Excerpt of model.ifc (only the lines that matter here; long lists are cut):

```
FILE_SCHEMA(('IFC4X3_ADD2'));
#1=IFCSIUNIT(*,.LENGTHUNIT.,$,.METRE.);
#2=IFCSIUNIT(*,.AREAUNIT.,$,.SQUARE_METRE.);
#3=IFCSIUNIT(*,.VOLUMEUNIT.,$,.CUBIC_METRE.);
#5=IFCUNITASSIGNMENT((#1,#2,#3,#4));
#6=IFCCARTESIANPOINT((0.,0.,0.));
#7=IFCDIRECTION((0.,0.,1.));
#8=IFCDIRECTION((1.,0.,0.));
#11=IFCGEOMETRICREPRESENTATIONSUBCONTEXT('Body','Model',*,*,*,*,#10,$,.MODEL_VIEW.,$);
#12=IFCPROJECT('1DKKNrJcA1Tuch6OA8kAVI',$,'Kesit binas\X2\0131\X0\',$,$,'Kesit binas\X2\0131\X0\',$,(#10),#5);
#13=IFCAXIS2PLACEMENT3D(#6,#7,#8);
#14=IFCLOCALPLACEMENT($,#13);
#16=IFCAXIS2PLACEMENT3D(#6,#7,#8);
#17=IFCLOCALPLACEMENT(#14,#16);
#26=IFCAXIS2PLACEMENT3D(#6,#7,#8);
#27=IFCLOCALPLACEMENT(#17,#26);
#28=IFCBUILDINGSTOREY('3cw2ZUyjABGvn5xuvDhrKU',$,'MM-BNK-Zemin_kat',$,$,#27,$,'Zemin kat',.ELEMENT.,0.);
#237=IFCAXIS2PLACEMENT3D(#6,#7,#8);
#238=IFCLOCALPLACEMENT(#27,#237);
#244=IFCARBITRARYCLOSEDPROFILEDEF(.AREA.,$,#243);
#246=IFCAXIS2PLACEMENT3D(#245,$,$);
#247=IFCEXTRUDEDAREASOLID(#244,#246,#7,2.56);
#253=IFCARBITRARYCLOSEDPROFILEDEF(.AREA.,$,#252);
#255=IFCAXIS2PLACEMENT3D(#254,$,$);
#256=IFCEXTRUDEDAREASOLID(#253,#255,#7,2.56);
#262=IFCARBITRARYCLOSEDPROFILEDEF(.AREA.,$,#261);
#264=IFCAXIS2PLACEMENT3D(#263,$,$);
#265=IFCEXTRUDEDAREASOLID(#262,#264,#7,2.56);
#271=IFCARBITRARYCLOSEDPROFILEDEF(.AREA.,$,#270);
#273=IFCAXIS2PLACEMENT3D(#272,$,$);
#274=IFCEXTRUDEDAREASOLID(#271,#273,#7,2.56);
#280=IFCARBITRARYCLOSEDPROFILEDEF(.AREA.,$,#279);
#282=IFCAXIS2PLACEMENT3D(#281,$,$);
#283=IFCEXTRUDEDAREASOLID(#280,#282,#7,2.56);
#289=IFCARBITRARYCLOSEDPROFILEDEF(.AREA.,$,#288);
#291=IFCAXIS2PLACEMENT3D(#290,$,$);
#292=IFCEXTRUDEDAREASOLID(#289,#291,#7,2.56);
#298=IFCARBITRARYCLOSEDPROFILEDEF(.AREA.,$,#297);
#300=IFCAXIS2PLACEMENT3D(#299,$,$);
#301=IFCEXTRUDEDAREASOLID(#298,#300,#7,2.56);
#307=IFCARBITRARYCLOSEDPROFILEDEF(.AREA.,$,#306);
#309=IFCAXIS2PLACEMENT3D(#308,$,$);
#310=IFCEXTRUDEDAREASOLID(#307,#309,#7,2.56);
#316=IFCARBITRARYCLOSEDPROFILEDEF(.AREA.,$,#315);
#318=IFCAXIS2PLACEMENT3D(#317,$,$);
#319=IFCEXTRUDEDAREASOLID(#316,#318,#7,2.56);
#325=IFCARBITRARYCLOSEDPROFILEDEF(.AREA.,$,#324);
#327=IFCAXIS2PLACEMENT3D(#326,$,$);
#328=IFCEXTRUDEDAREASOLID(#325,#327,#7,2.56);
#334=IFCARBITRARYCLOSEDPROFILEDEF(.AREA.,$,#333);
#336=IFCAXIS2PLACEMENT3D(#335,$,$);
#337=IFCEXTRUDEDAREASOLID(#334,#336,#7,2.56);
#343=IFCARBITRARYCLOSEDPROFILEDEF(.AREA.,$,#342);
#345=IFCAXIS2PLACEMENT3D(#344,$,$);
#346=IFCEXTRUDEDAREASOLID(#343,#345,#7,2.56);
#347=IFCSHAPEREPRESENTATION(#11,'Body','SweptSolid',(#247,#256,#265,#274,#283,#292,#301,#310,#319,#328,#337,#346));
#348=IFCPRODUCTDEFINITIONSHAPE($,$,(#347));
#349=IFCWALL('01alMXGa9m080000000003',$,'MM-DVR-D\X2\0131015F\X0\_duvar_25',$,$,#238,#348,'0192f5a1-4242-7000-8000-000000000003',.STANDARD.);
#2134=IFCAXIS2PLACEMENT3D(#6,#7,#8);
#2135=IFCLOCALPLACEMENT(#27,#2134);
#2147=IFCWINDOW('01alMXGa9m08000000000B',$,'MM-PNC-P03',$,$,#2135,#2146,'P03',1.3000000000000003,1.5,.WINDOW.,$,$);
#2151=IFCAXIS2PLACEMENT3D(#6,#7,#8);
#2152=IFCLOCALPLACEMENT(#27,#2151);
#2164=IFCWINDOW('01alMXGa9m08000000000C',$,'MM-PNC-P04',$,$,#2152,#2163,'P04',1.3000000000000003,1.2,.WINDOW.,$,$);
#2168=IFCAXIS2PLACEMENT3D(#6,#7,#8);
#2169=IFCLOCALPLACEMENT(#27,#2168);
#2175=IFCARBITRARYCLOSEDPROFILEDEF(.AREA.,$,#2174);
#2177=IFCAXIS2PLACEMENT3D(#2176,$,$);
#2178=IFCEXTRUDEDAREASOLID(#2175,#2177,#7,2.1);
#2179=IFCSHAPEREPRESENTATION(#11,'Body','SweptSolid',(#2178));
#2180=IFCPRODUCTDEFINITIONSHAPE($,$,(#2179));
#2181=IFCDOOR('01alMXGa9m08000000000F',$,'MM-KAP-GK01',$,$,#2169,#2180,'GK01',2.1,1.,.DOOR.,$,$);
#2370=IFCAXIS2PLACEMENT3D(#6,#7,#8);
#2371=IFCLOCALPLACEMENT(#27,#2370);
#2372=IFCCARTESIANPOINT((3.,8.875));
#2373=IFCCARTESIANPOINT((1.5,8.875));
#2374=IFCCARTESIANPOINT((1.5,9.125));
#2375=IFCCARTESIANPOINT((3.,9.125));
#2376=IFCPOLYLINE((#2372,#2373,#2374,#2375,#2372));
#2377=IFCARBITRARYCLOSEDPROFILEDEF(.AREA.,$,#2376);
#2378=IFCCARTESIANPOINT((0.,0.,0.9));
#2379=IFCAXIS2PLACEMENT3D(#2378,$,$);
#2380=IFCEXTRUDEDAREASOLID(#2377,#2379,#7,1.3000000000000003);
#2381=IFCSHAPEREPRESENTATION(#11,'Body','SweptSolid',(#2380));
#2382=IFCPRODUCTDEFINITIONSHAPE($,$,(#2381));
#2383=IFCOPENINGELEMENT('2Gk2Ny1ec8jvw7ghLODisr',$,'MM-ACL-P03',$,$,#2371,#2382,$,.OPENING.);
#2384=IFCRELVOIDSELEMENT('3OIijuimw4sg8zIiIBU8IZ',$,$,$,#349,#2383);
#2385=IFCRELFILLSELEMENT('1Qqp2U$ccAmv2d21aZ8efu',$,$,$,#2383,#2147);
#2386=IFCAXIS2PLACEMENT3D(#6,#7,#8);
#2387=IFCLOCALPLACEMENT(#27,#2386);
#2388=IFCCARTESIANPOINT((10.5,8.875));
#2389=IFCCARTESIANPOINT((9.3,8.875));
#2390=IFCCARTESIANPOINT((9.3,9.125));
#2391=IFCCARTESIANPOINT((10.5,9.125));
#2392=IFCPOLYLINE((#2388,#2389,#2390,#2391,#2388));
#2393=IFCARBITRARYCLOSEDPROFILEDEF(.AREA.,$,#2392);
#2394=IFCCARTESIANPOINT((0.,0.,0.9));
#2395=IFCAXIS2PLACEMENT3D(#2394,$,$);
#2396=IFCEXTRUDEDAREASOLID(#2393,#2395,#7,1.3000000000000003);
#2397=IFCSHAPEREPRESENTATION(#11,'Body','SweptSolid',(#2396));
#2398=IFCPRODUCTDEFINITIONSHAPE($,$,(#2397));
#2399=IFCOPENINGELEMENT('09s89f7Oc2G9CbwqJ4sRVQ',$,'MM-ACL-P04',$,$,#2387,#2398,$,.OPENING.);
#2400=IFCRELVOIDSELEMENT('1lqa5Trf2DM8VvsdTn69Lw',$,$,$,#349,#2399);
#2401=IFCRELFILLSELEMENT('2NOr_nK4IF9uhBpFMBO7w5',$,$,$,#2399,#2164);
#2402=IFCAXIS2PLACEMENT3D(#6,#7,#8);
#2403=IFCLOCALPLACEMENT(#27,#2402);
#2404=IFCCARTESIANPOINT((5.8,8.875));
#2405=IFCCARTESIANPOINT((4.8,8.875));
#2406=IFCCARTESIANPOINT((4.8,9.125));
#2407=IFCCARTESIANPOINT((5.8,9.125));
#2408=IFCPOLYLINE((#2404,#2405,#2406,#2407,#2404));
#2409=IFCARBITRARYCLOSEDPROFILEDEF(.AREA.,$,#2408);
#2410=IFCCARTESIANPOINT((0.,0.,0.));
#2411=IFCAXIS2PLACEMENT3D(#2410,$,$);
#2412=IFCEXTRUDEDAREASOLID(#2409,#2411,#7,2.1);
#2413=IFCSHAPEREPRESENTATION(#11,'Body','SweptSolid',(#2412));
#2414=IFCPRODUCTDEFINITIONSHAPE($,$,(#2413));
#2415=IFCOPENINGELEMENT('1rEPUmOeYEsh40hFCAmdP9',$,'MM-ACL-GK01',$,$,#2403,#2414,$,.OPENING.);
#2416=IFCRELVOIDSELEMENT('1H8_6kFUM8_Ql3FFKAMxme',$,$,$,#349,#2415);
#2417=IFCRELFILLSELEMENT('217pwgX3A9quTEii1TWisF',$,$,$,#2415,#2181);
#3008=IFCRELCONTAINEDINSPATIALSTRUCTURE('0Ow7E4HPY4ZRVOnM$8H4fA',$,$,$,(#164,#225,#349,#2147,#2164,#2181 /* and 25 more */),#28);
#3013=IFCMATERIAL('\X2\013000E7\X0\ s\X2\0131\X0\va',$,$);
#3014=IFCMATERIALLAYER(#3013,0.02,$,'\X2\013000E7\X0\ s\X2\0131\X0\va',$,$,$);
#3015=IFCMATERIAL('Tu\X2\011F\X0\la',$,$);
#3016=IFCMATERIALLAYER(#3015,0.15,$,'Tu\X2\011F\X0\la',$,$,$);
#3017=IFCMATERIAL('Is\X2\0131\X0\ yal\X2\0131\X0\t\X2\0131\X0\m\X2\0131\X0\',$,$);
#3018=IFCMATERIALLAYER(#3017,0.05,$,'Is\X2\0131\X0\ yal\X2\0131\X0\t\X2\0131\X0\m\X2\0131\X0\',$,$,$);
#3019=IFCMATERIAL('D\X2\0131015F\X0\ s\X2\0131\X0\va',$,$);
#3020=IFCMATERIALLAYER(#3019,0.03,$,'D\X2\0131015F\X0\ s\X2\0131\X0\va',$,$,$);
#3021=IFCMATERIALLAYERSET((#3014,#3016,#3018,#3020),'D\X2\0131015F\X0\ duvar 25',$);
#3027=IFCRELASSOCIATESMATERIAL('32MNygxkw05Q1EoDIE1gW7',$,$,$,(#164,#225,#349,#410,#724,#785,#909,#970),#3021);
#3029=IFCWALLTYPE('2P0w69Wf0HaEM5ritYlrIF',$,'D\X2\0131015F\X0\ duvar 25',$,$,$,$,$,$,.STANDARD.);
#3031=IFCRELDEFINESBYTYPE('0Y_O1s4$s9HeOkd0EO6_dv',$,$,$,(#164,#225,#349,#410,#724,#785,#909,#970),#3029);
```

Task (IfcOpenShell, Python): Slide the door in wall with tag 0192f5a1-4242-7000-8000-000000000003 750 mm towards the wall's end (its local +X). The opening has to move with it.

```python
import ifcopenshell
import ifcopenshell.api.geometry
import ifcopenshell.util.placement
import ifcopenshell.util.unit

model = ifcopenshell.open("model.ifc")
unit_scale = ifcopenshell.util.unit.calculate_unit_scale(model)

door = model.by_guid("01alMXGa9m08000000000F")
opening = door.FillsVoids[0].RelatingOpeningElement
wall = opening.VoidsElements[0].RelatingBuildingElement

wall_matrix = ifcopenshell.util.placement.get_local_placement(wall.ObjectPlacement)
shift = wall_matrix[:3, 0] * 0.75 / unit_scale
before = ifcopenshell.util.placement.get_local_placement(door.ObjectPlacement)[:3, 3].copy()

# The door is not placed relative to its opening, so move both.
for product in (opening, door):
    matrix = ifcopenshell.util.placement.get_local_placement(product.ObjectPlacement)
    matrix[:3, 3] += shift
    ifcopenshell.api.geometry.edit_object_placement(model, product=product, matrix=matrix, is_si=False)

after = ifcopenshell.util.placement.get_local_placement(door.ObjectPlacement)[:3, 3]
print("door moved by", (after - before).round(3) + 0.0)

model.write("model_v2.ifc")
```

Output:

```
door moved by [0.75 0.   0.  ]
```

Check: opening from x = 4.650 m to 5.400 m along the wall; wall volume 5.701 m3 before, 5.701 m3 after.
